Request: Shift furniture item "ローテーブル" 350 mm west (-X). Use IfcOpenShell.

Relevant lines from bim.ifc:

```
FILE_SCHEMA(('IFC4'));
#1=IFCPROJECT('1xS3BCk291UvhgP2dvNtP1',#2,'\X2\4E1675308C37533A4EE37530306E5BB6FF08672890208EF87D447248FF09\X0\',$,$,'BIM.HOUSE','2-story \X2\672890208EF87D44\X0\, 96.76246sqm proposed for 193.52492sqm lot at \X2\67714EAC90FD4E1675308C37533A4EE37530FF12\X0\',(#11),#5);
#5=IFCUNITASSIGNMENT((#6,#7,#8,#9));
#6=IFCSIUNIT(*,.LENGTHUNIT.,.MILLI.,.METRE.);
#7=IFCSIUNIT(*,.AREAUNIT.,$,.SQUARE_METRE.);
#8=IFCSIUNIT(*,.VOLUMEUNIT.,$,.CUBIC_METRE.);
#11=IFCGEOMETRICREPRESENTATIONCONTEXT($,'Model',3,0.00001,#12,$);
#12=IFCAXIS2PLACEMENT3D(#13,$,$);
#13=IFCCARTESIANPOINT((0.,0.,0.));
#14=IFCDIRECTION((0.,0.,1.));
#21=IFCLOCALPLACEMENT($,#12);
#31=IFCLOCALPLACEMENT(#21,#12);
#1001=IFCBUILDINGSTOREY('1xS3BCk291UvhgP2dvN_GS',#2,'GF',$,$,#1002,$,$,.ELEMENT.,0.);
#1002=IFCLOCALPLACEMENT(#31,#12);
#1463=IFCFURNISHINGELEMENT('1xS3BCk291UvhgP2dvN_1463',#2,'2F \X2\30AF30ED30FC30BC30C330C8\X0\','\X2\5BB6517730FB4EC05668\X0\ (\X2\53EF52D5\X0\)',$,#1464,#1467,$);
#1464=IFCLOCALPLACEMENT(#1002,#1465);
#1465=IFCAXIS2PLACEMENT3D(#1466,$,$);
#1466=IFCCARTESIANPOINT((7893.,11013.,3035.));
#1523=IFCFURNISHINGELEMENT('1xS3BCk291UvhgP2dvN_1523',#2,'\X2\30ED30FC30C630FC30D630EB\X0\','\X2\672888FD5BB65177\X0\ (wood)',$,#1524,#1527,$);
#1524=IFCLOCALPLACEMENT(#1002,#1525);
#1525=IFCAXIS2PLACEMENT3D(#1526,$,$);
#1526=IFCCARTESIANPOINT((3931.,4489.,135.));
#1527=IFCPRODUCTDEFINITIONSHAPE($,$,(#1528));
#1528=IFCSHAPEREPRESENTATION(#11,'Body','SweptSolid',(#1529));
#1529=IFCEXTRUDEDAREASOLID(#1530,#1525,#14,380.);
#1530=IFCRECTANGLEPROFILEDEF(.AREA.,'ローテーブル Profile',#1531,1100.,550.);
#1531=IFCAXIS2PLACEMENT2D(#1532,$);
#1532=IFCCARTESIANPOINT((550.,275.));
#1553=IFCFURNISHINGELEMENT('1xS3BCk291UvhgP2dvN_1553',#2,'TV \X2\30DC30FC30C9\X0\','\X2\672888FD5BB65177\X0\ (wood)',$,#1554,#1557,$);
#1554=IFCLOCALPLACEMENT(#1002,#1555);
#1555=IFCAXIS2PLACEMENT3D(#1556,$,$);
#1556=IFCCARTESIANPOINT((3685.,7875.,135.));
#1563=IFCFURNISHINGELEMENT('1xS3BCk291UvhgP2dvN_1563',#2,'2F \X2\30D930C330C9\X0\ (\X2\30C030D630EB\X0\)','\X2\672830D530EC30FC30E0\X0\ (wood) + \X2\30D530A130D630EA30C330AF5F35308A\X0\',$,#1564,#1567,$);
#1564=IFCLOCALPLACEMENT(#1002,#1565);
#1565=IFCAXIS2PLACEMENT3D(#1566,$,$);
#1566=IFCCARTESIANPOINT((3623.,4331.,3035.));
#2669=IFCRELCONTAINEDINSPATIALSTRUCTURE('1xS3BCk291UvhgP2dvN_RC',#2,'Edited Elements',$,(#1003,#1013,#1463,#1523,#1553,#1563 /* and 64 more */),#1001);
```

```python
import ifcopenshell
import ifcopenshell.api.geometry
import ifcopenshell.util.placement
import ifcopenshell.util.unit

model = ifcopenshell.open("bim.ifc")
unit_scale = ifcopenshell.util.unit.calculate_unit_scale(model)

item = model.by_guid("1xS3BCk291UvhgP2dvN_1523")
matrix = ifcopenshell.util.placement.get_local_placement(item.ObjectPlacement)
matrix[0, 3] -= 0.35 / unit_scale
ifcopenshell.api.geometry.edit_object_placement(model, product=item, matrix=matrix, is_si=False)

print(ifcopenshell.util.placement.get_local_placement(item.ObjectPlacement).round(3) + 0.0)

model.write("bim_edited.ifc")
```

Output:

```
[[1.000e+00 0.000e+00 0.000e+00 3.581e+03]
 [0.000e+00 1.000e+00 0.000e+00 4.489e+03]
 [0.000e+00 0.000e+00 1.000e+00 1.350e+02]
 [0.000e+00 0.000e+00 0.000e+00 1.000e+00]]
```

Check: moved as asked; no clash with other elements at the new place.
